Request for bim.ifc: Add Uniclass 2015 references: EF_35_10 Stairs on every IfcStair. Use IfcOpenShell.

First a look at what the model holds.

```python
import ifcopenshell

model = ifcopenshell.open("bim.ifc")
print(model.schema)
print("classifications:", [c.Name for c in model.by_type("IfcClassification")])
for ifc_class in ("IfcDoor", "IfcRoof", "IfcStair", "IfcWall", "IfcWindow"):
    print(ifc_class, len(model.by_type(ifc_class)))
```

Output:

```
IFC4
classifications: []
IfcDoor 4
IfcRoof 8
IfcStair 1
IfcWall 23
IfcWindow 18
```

```python
import ifcopenshell
import ifcopenshell.api.classification

model = ifcopenshell.open("bim.ifc")

system = ifcopenshell.api.classification.add_classification(model, classification="Uniclass 2015")

codes = {
    "IfcStair": ("EF_35_10", "Stairs"),
}
for ifc_class, (code, name) in codes.items():
    products = model.by_type(ifc_class)
    ifcopenshell.api.classification.add_reference(
        model, products=products, classification=system, identification=code, name=name
    )
    print(code, len(products))

model.write("bim_v2.ifc")
```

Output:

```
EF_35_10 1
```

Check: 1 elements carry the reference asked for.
